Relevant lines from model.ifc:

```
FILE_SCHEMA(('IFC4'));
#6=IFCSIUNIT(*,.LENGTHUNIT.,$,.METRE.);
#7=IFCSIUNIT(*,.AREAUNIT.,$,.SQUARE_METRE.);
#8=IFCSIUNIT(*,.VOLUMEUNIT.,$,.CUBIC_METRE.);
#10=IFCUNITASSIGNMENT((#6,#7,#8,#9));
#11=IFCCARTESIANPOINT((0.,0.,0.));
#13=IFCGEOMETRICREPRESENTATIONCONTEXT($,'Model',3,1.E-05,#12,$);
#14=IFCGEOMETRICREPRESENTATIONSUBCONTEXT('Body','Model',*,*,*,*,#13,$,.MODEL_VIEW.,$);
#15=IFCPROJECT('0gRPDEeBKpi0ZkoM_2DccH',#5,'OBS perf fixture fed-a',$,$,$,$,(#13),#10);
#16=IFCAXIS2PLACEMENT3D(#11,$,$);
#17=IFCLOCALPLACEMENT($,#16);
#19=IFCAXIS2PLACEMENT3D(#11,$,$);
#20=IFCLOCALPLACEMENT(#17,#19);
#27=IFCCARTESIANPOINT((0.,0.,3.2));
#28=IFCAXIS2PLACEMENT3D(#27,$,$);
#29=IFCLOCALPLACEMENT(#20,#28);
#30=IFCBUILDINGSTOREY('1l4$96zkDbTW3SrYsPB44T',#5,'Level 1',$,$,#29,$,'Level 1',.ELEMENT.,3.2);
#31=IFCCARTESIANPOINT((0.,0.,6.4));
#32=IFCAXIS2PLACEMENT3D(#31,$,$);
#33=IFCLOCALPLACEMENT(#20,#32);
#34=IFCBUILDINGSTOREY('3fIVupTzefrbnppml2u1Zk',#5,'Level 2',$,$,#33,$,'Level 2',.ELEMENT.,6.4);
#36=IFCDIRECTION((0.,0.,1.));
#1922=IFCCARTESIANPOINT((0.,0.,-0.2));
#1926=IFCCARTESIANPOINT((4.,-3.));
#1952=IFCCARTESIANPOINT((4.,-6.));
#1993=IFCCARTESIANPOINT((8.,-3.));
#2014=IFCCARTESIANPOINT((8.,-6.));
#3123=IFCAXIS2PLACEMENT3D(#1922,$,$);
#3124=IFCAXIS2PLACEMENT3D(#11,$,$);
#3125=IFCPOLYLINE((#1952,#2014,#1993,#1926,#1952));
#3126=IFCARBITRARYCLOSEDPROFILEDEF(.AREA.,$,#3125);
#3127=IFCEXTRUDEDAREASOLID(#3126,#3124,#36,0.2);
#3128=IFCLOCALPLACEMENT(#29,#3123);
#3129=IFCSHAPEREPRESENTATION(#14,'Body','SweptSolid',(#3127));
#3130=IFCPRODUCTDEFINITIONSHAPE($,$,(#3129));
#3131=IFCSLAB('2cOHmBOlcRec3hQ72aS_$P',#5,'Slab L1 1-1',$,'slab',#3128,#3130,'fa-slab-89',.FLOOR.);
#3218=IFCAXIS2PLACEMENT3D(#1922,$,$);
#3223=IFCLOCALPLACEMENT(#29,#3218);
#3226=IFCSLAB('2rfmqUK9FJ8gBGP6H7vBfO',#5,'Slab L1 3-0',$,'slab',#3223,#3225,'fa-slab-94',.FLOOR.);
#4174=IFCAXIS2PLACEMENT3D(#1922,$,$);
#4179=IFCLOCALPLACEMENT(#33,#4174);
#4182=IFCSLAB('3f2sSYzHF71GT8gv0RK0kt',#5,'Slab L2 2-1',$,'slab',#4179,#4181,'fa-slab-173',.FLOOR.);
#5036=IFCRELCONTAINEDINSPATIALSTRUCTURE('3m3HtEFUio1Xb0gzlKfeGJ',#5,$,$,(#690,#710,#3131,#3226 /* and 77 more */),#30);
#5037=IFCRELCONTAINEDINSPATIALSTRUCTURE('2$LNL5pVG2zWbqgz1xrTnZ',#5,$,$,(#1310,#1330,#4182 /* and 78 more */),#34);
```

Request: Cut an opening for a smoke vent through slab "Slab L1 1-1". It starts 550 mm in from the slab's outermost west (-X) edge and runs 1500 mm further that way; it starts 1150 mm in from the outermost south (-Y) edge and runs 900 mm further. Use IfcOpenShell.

```python
import numpy as np
import ifcopenshell
import ifcopenshell.api.feature
import ifcopenshell.api.geometry
import ifcopenshell.api.root
import ifcopenshell.geom
import ifcopenshell.util.placement
import ifcopenshell.util.representation
import ifcopenshell.util.shape
import ifcopenshell.util.unit

model = ifcopenshell.open("model.ifc")
unit_scale = ifcopenshell.util.unit.calculate_unit_scale(model)
settings = ifcopenshell.geom.settings()


def volume(element):
    """Net volume in cubic metres, openings subtracted."""
    shape = ifcopenshell.geom.create_shape(settings, element)
    return ifcopenshell.util.shape.get_volume(shape.geometry)


slab = model.by_guid("2cOHmBOlcRec3hQ72aS_$P")
before = volume(slab)

# Extent in the slab's own axes, in metres. The edges named are its -X and -Y sides.
slab_shape = ifcopenshell.geom.create_shape(settings, slab)
vertices = ifcopenshell.util.shape.get_vertices(slab_shape.geometry)
x_min, y_min, bottom = vertices.min(axis=0)
top = vertices[:, 2].max()

opening = ifcopenshell.api.root.create_entity(model, ifc_class="IfcOpeningElement", name="Smoke vent opening", predefined_type="OPENING")
context = ifcopenshell.util.representation.get_context(model, "Model", "Body", "MODEL_VIEW")
width, depth = 1.5, 0.9
outline = [(0.0, 0.0), (width, 0.0), (width, depth), (0.0, depth), (0.0, 0.0)]
# Overshoot both faces by 50 mm so the cut is clean.
shape = ifcopenshell.api.geometry.add_slab_representation(
    model, context=context, depth=top - bottom + 0.1, polyline=outline
)
ifcopenshell.api.geometry.assign_representation(model, product=opening, representation=shape)

matrix = ifcopenshell.util.placement.get_local_placement(slab.ObjectPlacement)
matrix[:, 3] = matrix @ np.append(np.array([x_min + 0.55, y_min + 1.15, bottom - 0.05]) / unit_scale, 1.0)
ifcopenshell.api.geometry.edit_object_placement(model, product=opening, matrix=matrix, is_si=False)
ifcopenshell.api.feature.add_feature(model, feature=opening, element=slab)

after = volume(slab)

print(f"slab volume {before:.3f} -> {after:.3f} m3")

model.write("model_v2.ifc")
```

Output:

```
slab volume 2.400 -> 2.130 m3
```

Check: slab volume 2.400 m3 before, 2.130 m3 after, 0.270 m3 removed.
